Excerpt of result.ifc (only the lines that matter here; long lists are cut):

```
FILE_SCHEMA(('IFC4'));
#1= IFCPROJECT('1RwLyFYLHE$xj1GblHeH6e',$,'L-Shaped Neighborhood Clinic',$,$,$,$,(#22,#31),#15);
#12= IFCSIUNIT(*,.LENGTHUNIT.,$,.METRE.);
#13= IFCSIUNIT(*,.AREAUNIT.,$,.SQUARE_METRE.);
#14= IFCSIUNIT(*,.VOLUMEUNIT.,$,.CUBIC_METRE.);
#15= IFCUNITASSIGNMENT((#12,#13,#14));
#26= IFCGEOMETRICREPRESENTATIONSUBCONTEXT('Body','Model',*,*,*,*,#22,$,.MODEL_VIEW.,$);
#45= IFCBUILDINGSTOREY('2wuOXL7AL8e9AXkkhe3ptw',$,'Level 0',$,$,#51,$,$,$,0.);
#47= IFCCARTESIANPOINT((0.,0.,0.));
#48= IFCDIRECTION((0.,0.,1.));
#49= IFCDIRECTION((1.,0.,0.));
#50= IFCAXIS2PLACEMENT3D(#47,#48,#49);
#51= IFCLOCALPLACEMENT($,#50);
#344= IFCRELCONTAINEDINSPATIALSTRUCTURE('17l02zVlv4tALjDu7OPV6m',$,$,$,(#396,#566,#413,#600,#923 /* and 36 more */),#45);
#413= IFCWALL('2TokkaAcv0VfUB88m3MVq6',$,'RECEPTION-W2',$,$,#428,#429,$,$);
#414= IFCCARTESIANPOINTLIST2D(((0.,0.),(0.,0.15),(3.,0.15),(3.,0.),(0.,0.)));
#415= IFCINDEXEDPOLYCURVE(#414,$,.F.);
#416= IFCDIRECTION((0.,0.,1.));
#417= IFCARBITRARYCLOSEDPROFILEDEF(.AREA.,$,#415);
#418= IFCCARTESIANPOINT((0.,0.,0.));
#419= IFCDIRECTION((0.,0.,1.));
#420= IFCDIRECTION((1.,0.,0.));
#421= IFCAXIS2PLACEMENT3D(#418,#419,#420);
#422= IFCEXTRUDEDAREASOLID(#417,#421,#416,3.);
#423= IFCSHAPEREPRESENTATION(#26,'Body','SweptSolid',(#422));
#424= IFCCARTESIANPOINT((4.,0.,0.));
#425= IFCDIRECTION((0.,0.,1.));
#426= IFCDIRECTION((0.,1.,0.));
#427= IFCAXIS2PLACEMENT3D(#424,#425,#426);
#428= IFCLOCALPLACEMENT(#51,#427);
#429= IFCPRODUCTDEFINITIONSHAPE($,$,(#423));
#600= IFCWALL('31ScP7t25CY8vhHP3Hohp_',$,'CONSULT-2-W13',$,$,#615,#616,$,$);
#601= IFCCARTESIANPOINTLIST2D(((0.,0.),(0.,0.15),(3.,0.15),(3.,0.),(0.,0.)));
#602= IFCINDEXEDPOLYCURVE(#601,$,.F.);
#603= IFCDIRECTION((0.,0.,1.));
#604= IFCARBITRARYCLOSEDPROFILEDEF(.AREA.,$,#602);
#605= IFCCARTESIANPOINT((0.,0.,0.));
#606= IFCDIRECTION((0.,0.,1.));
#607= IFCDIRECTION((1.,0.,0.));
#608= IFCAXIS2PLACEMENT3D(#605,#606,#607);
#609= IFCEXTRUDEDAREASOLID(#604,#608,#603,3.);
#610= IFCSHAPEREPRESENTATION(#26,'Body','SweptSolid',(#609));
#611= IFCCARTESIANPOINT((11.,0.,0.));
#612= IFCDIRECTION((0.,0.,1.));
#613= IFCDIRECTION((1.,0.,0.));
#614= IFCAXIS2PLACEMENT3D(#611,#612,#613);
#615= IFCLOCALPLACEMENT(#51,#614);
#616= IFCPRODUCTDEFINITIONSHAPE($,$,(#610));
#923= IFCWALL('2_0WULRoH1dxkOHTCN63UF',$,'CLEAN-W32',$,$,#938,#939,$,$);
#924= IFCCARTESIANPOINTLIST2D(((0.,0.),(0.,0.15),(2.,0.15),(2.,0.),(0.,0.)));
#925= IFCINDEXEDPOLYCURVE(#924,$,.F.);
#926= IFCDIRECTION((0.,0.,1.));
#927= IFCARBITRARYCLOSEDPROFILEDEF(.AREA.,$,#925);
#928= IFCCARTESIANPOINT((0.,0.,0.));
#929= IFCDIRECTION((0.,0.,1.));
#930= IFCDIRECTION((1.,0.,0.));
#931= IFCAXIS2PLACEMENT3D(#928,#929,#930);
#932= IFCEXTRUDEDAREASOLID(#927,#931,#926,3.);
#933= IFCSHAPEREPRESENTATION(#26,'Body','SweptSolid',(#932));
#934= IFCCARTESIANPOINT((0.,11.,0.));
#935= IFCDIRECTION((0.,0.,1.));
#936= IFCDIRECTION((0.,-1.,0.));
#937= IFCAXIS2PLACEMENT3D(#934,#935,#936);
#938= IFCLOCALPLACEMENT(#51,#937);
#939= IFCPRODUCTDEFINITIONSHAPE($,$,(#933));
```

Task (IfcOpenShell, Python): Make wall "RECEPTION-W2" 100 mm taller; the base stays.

```python
import ifcopenshell
import ifcopenshell.geom
import ifcopenshell.util.representation
import ifcopenshell.util.shape
import ifcopenshell.util.unit

model = ifcopenshell.open("result.ifc")
unit_scale = ifcopenshell.util.unit.calculate_unit_scale(model)
settings = ifcopenshell.geom.settings()


def volume(element):
    """Net volume in cubic metres, openings subtracted."""
    shape = ifcopenshell.geom.create_shape(settings, element)
    return ifcopenshell.util.shape.get_volume(shape.geometry)


wall = model.by_guid("2TokkaAcv0VfUB88m3MVq6")
before = volume(wall)

body = ifcopenshell.util.representation.get_representation(wall, "Model", "Body")
solid = body.Items[0]
old_height = solid.Depth
solid.Depth += 0.1 / unit_scale
after = volume(wall)

print(f"height {old_height:g} -> {solid.Depth:g}, volume {before:.3f} -> {after:.3f} m3")

model.write("result_updated.ifc")
```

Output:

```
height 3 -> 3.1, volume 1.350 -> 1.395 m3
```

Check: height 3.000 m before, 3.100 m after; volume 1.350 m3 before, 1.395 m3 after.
